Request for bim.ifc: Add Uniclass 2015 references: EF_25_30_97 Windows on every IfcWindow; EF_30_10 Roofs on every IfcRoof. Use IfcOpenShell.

First a look at what the model holds.

```python
import ifcopenshell

model = ifcopenshell.open("bim.ifc")
print(model.schema)
print("classifications:", [c.Name for c in model.by_type("IfcClassification")])
for ifc_class in ("IfcDoor", "IfcRoof", "IfcStair", "IfcWall", "IfcWindow"):
    print(ifc_class, len(model.by_type(ifc_class)))
```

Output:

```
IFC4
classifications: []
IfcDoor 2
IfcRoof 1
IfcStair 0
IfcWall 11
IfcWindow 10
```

```python
import ifcopenshell
import ifcopenshell.api.classification

model = ifcopenshell.open("bim.ifc")

system = ifcopenshell.api.classification.add_classification(model, classification="Uniclass 2015")

codes = {
    "IfcWindow": ("EF_25_30_97", "Windows"),
    "IfcRoof": ("EF_30_10", "Roofs"),
}
for ifc_class, (code, name) in codes.items():
    products = model.by_type(ifc_class)
    ifcopenshell.api.classification.add_reference(
        model, products=products, classification=system, identification=code, name=name
    )
    print(code, len(products))

model.write("bim_v2.ifc")
```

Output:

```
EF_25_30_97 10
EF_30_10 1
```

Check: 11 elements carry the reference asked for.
